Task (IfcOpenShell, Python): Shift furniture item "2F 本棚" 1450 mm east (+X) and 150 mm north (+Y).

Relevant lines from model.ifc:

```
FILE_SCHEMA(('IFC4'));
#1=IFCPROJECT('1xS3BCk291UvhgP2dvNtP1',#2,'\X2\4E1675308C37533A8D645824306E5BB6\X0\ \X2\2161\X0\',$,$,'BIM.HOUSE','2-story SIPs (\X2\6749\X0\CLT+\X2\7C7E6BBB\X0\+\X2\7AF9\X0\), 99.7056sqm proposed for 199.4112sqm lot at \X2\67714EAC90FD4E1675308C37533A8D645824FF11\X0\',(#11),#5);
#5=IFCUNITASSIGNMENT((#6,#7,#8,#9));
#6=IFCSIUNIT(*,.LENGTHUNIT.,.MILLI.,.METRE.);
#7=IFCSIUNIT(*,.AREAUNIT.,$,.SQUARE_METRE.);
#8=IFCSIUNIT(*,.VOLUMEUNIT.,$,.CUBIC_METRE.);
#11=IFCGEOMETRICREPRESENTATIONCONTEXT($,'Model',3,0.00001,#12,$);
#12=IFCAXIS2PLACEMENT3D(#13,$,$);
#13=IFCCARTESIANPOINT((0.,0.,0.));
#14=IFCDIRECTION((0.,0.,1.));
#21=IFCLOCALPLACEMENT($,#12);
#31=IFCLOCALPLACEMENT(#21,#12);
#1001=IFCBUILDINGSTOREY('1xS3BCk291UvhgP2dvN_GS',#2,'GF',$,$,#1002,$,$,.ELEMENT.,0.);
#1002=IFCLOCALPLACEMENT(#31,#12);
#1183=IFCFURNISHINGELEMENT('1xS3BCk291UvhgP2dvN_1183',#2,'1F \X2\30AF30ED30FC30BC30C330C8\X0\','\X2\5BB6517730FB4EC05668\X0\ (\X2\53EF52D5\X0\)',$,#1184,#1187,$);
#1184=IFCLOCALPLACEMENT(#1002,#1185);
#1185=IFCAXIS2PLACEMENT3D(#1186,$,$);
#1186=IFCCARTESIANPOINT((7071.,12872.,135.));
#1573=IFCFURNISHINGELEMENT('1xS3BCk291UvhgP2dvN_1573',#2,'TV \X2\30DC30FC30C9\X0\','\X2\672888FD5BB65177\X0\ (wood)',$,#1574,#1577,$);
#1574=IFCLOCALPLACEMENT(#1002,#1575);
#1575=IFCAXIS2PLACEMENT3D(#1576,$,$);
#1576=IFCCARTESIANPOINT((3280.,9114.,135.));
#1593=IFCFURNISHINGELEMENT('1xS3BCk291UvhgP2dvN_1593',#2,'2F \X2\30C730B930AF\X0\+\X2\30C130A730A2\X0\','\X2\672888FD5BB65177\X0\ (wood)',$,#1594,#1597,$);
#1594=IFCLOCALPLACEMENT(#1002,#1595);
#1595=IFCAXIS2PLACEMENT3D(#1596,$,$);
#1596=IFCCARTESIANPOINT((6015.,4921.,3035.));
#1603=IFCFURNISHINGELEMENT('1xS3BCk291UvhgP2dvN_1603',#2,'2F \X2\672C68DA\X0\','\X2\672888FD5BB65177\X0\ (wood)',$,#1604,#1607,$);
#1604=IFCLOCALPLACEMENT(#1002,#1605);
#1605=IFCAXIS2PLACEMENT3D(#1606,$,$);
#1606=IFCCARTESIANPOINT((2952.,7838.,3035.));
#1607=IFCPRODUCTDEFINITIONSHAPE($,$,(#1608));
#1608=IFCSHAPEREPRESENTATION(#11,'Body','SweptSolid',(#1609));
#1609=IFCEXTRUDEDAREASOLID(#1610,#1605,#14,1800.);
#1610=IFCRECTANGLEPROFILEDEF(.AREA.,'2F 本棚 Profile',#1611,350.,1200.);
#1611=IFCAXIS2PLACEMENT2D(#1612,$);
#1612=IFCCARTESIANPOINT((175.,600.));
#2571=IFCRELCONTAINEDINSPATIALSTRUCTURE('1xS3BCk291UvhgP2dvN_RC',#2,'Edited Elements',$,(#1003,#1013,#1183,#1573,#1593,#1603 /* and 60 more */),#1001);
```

```python
import ifcopenshell
import ifcopenshell.api.geometry
import ifcopenshell.util.placement

model = ifcopenshell.open("model.ifc")

item = model.by_id(1603)
matrix = ifcopenshell.util.placement.get_local_placement(item.ObjectPlacement)
matrix[0, 3] += 1450.0
matrix[1, 3] += 150.0
ifcopenshell.api.geometry.edit_object_placement(model, product=item, matrix=matrix, is_si=False)

print(ifcopenshell.util.placement.get_local_placement(item.ObjectPlacement).round(3) + 0.0)

model.write("model_updated.ifc")
```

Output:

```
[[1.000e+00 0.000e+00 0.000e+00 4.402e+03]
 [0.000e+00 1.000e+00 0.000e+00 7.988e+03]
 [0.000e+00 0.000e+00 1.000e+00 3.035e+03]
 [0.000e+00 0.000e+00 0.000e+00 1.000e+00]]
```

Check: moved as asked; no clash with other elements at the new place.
